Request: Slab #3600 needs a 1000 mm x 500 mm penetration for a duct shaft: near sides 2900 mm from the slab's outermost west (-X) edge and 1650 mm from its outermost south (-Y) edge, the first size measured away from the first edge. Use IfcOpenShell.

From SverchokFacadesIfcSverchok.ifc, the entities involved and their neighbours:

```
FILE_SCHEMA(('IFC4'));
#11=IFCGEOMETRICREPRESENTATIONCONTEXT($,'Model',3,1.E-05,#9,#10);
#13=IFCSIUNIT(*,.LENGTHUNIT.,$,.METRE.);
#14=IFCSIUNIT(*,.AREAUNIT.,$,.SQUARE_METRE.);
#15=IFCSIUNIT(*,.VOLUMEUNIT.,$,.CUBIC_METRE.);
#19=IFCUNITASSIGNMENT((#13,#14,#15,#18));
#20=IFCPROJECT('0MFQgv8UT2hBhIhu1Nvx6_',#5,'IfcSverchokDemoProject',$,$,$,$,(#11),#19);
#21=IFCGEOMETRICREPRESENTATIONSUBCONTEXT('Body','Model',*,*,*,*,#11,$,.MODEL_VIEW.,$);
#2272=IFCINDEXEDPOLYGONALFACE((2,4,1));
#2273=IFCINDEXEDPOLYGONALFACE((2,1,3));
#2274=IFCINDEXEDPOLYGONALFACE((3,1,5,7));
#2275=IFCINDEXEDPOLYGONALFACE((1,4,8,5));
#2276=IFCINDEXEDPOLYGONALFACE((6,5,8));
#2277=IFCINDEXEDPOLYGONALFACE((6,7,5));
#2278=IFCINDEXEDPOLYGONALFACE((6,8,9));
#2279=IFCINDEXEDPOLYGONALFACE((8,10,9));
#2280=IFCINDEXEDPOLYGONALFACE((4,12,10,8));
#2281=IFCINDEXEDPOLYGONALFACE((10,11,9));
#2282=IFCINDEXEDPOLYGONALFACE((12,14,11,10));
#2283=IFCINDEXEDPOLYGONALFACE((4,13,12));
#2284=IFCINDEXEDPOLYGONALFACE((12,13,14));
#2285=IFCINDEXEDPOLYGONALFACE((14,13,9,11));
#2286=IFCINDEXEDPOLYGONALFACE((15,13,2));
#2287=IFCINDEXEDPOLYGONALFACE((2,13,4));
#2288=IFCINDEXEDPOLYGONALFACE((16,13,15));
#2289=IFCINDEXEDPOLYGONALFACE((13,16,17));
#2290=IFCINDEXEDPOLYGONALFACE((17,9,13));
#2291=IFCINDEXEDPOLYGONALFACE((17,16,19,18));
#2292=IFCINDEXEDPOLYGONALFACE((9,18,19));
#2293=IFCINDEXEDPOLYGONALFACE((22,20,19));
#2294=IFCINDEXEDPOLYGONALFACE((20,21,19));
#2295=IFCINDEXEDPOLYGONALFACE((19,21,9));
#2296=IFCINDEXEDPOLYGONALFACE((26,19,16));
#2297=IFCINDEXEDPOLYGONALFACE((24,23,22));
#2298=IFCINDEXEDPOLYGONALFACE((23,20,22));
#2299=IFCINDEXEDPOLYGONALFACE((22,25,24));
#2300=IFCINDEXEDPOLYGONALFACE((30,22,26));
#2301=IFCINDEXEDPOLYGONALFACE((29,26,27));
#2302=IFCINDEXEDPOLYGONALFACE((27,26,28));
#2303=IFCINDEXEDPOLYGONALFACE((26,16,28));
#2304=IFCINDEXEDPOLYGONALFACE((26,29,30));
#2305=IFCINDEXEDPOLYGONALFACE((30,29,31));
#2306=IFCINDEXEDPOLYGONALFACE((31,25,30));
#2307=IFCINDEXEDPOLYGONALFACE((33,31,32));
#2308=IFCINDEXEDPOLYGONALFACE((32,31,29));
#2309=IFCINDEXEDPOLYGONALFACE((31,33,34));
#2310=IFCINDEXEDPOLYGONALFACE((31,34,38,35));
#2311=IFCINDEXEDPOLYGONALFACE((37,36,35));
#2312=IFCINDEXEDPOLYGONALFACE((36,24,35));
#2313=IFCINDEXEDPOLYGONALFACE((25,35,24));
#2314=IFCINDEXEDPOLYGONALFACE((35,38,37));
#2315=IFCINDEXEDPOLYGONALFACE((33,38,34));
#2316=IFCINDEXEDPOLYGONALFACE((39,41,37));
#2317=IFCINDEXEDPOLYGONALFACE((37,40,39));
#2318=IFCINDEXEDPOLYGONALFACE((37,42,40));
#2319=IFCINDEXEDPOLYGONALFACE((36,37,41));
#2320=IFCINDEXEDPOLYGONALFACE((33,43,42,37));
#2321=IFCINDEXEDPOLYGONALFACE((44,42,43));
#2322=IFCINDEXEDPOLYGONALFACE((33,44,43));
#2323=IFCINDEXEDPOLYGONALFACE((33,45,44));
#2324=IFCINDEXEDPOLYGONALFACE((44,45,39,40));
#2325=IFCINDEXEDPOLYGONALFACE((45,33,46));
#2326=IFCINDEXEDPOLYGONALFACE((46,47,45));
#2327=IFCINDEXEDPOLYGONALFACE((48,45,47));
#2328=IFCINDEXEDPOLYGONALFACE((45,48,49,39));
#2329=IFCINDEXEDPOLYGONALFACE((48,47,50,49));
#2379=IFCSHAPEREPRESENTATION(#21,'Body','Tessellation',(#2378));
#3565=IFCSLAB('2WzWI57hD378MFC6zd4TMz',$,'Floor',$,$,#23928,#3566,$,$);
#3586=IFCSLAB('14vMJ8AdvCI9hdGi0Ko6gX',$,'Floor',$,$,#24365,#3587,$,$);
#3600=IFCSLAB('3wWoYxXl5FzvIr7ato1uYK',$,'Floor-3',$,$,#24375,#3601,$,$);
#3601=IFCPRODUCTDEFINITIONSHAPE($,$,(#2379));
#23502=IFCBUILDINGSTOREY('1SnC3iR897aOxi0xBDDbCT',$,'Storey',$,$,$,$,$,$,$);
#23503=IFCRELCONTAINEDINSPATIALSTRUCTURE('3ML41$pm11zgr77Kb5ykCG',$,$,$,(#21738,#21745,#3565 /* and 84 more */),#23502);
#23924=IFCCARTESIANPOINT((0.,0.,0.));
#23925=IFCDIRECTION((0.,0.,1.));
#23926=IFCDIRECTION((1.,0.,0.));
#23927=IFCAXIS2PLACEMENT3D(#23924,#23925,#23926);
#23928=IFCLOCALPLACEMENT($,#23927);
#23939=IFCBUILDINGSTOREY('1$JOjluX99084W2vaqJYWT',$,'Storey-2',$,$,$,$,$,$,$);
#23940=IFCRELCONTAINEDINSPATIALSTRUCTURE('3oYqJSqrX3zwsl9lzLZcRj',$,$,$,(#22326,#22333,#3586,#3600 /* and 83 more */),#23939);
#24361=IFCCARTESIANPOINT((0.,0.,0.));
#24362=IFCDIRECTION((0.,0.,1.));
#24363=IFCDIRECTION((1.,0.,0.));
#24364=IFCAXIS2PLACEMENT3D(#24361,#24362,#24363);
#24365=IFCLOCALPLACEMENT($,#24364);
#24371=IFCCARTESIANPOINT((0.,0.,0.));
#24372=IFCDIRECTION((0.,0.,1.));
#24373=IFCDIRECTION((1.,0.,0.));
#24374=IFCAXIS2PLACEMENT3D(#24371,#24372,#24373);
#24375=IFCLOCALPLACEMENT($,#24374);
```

```python
import numpy as np
import ifcopenshell
import ifcopenshell.api.feature
import ifcopenshell.api.geometry
import ifcopenshell.api.root
import ifcopenshell.geom
import ifcopenshell.util.placement
import ifcopenshell.util.representation
import ifcopenshell.util.shape
import ifcopenshell.util.unit

model = ifcopenshell.open("SverchokFacadesIfcSverchok.ifc")
unit_scale = ifcopenshell.util.unit.calculate_unit_scale(model)
settings = ifcopenshell.geom.settings()


def volume(element):
    """Net volume in cubic metres, openings subtracted."""
    shape = ifcopenshell.geom.create_shape(settings, element)
    return ifcopenshell.util.shape.get_volume(shape.geometry)


slab = model.by_id(3600)
before = volume(slab)

# Extent in the slab's own axes, in metres. The edges named are its -X and -Y sides.
slab_shape = ifcopenshell.geom.create_shape(settings, slab)
vertices = ifcopenshell.util.shape.get_vertices(slab_shape.geometry)
x_min, y_min, bottom = vertices.min(axis=0)
top = vertices[:, 2].max()

opening = ifcopenshell.api.root.create_entity(model, ifc_class="IfcOpeningElement", name="Duct shaft opening", predefined_type="OPENING")
context = ifcopenshell.util.representation.get_context(model, "Model", "Body", "MODEL_VIEW")
width, depth = 1, 0.5
outline = [(0.0, 0.0), (width, 0.0), (width, depth), (0.0, depth), (0.0, 0.0)]
# Overshoot both faces by 50 mm so the cut is clean.
shape = ifcopenshell.api.geometry.add_slab_representation(
    model, context=context, depth=top - bottom + 0.1, polyline=outline
)
ifcopenshell.api.geometry.assign_representation(model, product=opening, representation=shape)

matrix = ifcopenshell.util.placement.get_local_placement(slab.ObjectPlacement)
matrix[:, 3] = matrix @ np.append(np.array([x_min + 2.9, y_min + 1.65, bottom - 0.05]) / unit_scale, 1.0)
ifcopenshell.api.geometry.edit_object_placement(model, product=opening, matrix=matrix, is_si=False)
ifcopenshell.api.feature.add_feature(model, feature=opening, element=slab)

after = volume(slab)

print(f"slab volume {before:.3f} -> {after:.3f} m3")

model.write("SverchokFacadesIfcSverchok_edited.ifc")
```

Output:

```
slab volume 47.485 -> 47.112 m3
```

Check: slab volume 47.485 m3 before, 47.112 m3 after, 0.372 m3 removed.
